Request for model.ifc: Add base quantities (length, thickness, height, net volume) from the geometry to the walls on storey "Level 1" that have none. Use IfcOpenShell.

First a look at what the model holds.

```python
import ifcopenshell
import ifcopenshell.util.element
import ifcopenshell.util.unit

model = ifcopenshell.open("model.ifc")
print(model.schema)
for unit_type in ("LENGTHUNIT", "AREAUNIT", "VOLUMEUNIT"):
    print(unit_type, ifcopenshell.util.unit.calculate_unit_scale(model, unit_type))
storey = next(s for s in model.by_type("IfcBuildingStorey") if s.Name == "Level 1")
walls = [e for e in ifcopenshell.util.element.get_decomposition(storey) if e.is_a("IfcWall")]
for e in sorted(walls, key=lambda e: e.id()):
    print(e.id(), e.is_a(), e.Name, list(ifcopenshell.util.element.get_psets(e, qtos_only=True)), sep=" | ")
```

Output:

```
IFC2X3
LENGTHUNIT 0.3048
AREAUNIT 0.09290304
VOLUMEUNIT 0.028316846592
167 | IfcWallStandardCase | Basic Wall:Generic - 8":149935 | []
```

```python
import ifcopenshell
import ifcopenshell.api.pset
import ifcopenshell.geom
import ifcopenshell.util.element
import ifcopenshell.util.shape
import ifcopenshell.util.unit

model = ifcopenshell.open("model.ifc")
unit_scale = ifcopenshell.util.unit.calculate_unit_scale(model)
volume_scale = ifcopenshell.util.unit.calculate_unit_scale(model, "VOLUMEUNIT")
settings = ifcopenshell.geom.settings()

storey = next(s for s in model.by_type("IfcBuildingStorey") if s.Name == "Level 1")
walls = [e for e in ifcopenshell.util.element.get_decomposition(storey) if e.is_a("IfcWall")]

for e in sorted(walls, key=lambda e: e.id()):
    if ifcopenshell.util.element.get_psets(e, qtos_only=True, should_inherit=False):
        continue
    # Geometry comes back in metres, in the element's own axes.
    shape = ifcopenshell.geom.create_shape(settings, e)
    values = {
        "Length": ifcopenshell.util.shape.get_x(shape.geometry) / unit_scale,
        "Width": ifcopenshell.util.shape.get_y(shape.geometry) / unit_scale,
        "Height": ifcopenshell.util.shape.get_z(shape.geometry) / unit_scale,
        "NetVolume": ifcopenshell.util.shape.get_volume(shape.geometry) / volume_scale,
    }
    qto = ifcopenshell.api.pset.add_qto(model, product=e, name="BaseQuantities")
    ifcopenshell.api.pset.edit_qto(model, qto=qto, properties=values)
    print(e.id(), {k: round(v, 3) for k, v in values.items()})

model.write("model_v2.ifc")
```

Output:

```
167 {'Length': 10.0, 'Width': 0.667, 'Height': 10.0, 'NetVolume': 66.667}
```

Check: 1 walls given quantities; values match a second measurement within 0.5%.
